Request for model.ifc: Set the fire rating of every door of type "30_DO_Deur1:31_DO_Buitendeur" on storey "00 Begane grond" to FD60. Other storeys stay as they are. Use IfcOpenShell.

First a look at what the model holds.

```python
import ifcopenshell
import ifcopenshell.util.element

model = ifcopenshell.open("model.ifc")
print(model.schema)
storey = next(s for s in model.by_type("IfcBuildingStorey") if s.Name == "00 Begane grond")
doors = [e for e in ifcopenshell.util.element.get_decomposition(storey) if e.is_a("IfcDoor")]
seen = {}
for e in doors:
    element_type = ifcopenshell.util.element.get_type(e)
    key = (element_type.Name if element_type != e and element_type else None, ifcopenshell.util.element.get_pset(e, "Pset_DoorCommon", "FireRating"))
    seen[key] = seen.get(key, 0) + 1
for (name, value), count in sorted(seen.items(), key=str):
    print(count, "x", name, "|", value)
```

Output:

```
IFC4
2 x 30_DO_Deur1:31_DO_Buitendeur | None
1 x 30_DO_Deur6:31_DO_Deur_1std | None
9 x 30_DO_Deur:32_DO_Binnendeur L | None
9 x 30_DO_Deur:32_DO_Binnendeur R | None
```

```python
import ifcopenshell
import ifcopenshell.api.pset
import ifcopenshell.util.element

model = ifcopenshell.open("model.ifc")

storey = next(s for s in model.by_type("IfcBuildingStorey") if s.Name == "00 Begane grond")
doors = [e for e in ifcopenshell.util.element.get_decomposition(storey) if e.is_a("IfcDoor")]

count = 0
for e in doors:
    element_type = ifcopenshell.util.element.get_type(e)
    if element_type in (None, e) or element_type.Name != "30_DO_Deur1:31_DO_Buitendeur":
        continue
    # add_pset returns the element's existing set when there is one.
    pset = ifcopenshell.api.pset.add_pset(model, product=e, name="Pset_DoorCommon")
    ifcopenshell.api.pset.edit_pset(model, pset=pset, properties={"FireRating": "FD60"})
    count += 1

print(count, "doors updated")

model.write("model_updated.ifc")
```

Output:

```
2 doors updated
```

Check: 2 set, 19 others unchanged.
